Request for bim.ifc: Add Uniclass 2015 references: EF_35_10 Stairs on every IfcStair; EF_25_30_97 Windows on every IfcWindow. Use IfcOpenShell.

First a look at what the model holds.

```python
import ifcopenshell

model = ifcopenshell.open("bim.ifc")
print(model.schema)
print("classifications:", [c.Name for c in model.by_type("IfcClassification")])
for ifc_class in ("IfcDoor", "IfcRoof", "IfcStair", "IfcWall", "IfcWindow"):
    print(ifc_class, len(model.by_type(ifc_class)))
```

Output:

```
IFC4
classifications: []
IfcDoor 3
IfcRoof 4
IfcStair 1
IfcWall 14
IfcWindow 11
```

```python
import ifcopenshell
import ifcopenshell.api.classification

model = ifcopenshell.open("bim.ifc")

system = ifcopenshell.api.classification.add_classification(model, classification="Uniclass 2015")

codes = {
    "IfcStair": ("EF_35_10", "Stairs"),
    "IfcWindow": ("EF_25_30_97", "Windows"),
}
for ifc_class, (code, name) in codes.items():
    products = model.by_type(ifc_class)
    ifcopenshell.api.classification.add_reference(
        model, products=products, classification=system, identification=code, name=name
    )
    print(code, len(products))

model.write("bim_v2.ifc")
```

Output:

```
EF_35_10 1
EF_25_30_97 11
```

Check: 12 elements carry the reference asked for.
